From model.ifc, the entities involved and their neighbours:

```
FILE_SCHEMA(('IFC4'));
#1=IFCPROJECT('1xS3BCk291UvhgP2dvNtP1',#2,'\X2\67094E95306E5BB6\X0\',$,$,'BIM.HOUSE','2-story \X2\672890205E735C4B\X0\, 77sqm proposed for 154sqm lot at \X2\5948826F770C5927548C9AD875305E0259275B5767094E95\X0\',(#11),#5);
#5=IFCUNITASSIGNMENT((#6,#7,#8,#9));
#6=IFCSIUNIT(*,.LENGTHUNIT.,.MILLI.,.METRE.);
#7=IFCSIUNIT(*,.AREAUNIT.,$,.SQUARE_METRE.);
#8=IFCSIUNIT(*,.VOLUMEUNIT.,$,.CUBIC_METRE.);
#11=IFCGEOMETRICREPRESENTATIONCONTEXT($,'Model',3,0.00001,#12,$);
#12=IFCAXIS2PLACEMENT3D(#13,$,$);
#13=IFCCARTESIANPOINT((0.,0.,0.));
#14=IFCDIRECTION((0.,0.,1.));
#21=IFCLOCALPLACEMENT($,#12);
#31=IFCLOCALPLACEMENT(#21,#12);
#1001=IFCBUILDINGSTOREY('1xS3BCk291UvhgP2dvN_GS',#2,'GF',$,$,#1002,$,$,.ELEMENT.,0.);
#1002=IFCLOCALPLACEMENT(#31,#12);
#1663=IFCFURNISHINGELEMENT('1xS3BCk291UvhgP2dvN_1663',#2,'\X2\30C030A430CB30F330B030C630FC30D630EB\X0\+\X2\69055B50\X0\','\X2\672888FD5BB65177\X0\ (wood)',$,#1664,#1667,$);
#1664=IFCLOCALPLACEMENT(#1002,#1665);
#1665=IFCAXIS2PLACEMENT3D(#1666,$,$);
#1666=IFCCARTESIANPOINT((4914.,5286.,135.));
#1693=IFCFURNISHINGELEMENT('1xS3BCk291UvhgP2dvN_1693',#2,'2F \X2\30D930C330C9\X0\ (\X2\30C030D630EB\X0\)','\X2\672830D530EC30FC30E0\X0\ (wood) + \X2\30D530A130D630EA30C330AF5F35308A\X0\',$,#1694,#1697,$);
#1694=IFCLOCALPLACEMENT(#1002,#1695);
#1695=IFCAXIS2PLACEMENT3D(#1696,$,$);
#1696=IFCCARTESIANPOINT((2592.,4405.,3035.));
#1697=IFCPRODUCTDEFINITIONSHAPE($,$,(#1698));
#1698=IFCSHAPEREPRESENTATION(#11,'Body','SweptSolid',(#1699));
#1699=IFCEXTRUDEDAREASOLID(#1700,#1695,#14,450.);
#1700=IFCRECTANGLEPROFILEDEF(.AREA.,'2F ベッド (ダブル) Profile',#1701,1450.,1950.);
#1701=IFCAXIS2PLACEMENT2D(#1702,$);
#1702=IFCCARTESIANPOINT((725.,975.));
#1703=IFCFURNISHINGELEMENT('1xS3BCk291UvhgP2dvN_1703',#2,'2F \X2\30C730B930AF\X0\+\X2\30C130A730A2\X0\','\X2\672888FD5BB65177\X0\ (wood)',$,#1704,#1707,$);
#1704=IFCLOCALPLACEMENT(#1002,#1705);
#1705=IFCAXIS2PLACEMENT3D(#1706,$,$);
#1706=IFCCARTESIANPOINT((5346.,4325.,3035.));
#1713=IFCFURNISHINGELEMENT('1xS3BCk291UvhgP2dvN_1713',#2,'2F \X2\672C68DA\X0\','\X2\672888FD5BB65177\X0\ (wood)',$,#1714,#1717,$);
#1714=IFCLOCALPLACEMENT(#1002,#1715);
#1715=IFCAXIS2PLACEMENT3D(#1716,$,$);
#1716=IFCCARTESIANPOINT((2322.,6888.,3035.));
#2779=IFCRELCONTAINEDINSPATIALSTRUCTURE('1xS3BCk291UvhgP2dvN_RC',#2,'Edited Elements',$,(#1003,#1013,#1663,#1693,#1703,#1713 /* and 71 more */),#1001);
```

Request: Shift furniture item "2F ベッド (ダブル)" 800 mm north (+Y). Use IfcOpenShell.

```python
import ifcopenshell
import ifcopenshell.api.geometry
import ifcopenshell.util.placement
import ifcopenshell.util.unit

model = ifcopenshell.open("model.ifc")
unit_scale = ifcopenshell.util.unit.calculate_unit_scale(model)

item = model.by_id(1693)
matrix = ifcopenshell.util.placement.get_local_placement(item.ObjectPlacement)
matrix[1, 3] += 0.8 / unit_scale
ifcopenshell.api.geometry.edit_object_placement(model, product=item, matrix=matrix, is_si=False)

print(ifcopenshell.util.placement.get_local_placement(item.ObjectPlacement).round(3) + 0.0)

model.write("model_updated.ifc")
```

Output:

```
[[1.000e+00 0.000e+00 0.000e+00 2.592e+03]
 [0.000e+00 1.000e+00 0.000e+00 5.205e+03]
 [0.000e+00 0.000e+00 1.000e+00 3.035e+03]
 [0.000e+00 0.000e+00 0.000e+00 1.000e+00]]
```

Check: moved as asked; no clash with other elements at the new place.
